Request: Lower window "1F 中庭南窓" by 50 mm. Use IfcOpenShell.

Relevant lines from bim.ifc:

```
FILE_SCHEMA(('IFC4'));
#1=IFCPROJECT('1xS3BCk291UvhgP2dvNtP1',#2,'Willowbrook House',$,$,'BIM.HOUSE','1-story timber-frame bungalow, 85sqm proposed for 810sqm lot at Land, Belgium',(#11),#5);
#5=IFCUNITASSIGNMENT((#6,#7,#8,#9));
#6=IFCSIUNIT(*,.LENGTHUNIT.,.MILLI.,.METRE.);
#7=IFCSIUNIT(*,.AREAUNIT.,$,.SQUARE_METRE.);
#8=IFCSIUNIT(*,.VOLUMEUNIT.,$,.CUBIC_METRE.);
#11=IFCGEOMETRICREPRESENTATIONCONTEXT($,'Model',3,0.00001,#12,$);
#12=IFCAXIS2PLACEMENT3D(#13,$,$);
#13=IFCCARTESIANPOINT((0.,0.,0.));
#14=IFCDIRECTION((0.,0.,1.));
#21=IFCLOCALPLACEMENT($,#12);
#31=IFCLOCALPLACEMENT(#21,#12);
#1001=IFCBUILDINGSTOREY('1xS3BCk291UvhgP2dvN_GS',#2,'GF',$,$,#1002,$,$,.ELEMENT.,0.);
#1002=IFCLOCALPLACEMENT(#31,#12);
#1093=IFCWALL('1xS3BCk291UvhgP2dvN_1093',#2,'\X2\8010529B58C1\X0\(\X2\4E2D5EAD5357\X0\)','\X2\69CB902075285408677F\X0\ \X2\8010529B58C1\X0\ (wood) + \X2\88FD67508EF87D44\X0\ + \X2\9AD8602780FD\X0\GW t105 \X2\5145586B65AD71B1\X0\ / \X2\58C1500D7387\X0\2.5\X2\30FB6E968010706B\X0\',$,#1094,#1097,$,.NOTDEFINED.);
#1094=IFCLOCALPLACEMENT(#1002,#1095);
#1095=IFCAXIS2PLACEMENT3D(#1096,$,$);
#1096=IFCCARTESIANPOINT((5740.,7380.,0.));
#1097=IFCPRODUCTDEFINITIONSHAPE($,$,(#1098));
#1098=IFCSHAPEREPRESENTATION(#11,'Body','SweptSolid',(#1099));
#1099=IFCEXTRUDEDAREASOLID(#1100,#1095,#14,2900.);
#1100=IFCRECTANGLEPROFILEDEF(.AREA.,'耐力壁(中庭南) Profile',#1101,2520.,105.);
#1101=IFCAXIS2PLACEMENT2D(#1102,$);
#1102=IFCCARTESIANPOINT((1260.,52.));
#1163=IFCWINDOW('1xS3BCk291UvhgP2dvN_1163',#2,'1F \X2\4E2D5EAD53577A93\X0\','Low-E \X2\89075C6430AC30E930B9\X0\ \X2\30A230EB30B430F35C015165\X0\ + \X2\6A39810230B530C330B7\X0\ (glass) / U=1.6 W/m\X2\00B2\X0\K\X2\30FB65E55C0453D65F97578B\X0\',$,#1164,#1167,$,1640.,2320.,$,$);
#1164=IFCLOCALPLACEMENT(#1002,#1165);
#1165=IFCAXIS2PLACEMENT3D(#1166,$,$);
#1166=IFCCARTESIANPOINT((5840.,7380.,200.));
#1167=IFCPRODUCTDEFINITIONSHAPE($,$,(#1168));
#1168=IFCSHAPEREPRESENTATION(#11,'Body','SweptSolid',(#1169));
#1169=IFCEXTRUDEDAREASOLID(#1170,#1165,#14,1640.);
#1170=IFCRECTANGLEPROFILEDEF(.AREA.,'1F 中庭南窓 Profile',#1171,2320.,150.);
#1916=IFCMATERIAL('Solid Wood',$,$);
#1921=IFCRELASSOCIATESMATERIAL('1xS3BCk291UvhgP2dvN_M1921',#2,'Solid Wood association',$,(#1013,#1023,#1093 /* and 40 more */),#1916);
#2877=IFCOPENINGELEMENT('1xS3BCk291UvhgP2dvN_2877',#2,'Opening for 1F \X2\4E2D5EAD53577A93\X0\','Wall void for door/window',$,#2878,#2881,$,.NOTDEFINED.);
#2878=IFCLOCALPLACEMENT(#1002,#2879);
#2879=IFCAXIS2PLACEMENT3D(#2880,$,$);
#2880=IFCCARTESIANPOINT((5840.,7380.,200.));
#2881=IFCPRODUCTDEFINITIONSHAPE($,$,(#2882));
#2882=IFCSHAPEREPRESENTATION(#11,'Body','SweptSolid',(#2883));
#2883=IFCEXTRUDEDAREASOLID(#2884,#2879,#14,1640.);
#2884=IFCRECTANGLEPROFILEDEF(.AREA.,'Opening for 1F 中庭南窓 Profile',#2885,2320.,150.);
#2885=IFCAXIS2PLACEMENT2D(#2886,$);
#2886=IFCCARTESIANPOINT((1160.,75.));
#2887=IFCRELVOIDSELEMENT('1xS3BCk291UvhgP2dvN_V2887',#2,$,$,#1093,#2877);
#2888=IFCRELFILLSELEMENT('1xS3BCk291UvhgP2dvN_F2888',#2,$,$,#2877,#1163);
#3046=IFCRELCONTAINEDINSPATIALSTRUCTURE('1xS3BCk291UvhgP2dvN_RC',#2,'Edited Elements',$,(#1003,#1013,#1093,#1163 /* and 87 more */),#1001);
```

```python
import numpy as np
import ifcopenshell
import ifcopenshell.api.geometry
import ifcopenshell.util.placement
import ifcopenshell.util.unit

model = ifcopenshell.open("bim.ifc")
unit_scale = ifcopenshell.util.unit.calculate_unit_scale(model)

window = model.by_guid("1xS3BCk291UvhgP2dvN_1163")
opening = window.FillsVoids[0].RelatingOpeningElement
dz = -50.0

shift = np.array([0.0, 0.0, dz])
# The window is not placed relative to its opening, so move both.
for product in (opening, window):
    matrix = ifcopenshell.util.placement.get_local_placement(product.ObjectPlacement)
    matrix[:3, 3] += shift
    ifcopenshell.api.geometry.edit_object_placement(model, product=product, matrix=matrix, is_si=False)

print(f"moved by {dz * unit_scale:+.3f} m")

model.write("bim-out.ifc")
```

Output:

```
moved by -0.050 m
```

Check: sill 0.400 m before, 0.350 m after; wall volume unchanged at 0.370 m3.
